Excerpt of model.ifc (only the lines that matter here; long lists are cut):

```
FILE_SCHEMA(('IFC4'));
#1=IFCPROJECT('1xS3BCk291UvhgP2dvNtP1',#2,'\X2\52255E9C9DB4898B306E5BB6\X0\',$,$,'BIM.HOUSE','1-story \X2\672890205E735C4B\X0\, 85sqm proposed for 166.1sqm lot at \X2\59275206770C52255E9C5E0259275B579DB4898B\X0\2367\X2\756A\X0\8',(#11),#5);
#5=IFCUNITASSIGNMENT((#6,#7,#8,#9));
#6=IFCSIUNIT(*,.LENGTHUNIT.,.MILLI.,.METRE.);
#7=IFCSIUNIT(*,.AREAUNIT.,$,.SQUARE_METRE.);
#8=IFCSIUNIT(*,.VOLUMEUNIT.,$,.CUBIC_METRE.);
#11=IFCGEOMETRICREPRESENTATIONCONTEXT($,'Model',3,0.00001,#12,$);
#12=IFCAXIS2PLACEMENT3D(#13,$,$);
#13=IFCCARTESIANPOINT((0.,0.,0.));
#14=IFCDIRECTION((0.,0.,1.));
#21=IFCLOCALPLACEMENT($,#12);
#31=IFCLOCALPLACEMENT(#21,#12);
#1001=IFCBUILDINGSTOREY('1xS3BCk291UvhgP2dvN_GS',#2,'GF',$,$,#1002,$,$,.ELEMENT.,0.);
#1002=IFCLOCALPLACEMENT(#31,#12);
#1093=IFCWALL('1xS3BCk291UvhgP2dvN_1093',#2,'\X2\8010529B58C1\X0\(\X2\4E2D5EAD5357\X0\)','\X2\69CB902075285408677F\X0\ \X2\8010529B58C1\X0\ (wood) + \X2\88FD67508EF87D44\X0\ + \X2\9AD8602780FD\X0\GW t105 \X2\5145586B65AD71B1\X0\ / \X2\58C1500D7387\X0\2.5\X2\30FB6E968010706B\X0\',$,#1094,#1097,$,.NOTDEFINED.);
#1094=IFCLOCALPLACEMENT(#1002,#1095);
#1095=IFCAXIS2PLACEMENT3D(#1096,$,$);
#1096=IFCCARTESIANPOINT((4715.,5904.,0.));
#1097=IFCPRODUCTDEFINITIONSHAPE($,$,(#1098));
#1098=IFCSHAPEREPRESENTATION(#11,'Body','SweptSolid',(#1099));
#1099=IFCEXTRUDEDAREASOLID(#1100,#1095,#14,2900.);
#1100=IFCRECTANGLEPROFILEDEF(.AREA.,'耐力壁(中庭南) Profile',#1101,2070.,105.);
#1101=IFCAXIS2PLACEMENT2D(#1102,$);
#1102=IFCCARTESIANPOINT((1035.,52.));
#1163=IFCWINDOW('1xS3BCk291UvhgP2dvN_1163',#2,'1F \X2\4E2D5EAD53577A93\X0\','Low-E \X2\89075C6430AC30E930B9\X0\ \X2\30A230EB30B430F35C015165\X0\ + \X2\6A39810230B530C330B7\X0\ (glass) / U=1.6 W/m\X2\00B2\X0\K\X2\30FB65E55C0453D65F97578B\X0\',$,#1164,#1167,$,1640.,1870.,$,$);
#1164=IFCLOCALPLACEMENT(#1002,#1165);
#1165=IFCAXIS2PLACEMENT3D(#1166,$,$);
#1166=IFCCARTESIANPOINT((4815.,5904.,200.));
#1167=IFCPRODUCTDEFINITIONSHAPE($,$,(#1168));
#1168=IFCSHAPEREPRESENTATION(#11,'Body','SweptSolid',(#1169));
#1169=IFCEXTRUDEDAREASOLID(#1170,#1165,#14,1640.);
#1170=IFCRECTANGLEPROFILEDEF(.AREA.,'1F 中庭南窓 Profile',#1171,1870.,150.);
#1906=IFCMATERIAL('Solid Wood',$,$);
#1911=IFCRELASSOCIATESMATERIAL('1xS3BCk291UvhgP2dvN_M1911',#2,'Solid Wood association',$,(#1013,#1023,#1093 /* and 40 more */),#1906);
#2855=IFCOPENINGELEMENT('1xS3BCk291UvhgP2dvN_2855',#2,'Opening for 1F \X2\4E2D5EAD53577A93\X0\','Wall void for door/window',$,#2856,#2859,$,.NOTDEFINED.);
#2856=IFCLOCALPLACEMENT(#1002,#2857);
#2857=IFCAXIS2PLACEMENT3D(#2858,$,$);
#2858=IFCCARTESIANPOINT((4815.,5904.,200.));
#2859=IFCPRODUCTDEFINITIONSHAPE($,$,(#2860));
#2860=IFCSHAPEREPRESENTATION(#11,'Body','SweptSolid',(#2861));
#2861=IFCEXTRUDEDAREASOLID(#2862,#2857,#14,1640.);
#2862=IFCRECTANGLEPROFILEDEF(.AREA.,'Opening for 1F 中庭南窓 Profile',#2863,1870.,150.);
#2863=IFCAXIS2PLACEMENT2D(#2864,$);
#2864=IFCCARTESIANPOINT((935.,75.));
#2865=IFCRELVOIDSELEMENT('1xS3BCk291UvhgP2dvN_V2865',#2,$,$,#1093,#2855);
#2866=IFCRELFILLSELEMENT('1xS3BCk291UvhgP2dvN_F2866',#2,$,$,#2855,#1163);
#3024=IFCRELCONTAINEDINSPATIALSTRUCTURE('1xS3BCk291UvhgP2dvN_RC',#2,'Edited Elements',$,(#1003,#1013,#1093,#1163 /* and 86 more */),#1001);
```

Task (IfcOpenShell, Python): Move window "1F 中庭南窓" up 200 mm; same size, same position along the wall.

```python
import numpy as np
import ifcopenshell
import ifcopenshell.api.geometry
import ifcopenshell.util.placement
import ifcopenshell.util.unit

model = ifcopenshell.open("model.ifc")
unit_scale = ifcopenshell.util.unit.calculate_unit_scale(model)

window = model.by_guid("1xS3BCk291UvhgP2dvN_1163")
opening = window.FillsVoids[0].RelatingOpeningElement
dz = 200.0

shift = np.array([0.0, 0.0, dz])
# The window is not placed relative to its opening, so move both.
for product in (opening, window):
    matrix = ifcopenshell.util.placement.get_local_placement(product.ObjectPlacement)
    matrix[:3, 3] += shift
    ifcopenshell.api.geometry.edit_object_placement(model, product=product, matrix=matrix, is_si=False)

print(f"moved by {dz * unit_scale:+.3f} m")

model.write("model_updated.ifc")
```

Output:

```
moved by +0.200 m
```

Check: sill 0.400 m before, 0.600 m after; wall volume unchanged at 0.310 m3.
